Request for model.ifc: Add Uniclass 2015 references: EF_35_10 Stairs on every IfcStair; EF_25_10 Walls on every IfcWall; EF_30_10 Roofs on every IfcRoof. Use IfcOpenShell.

First a look at what the model holds.

```python
import ifcopenshell

model = ifcopenshell.open("model.ifc")
print(model.schema)
print("classifications:", [c.Name for c in model.by_type("IfcClassification")])
for ifc_class in ("IfcDoor", "IfcRoof", "IfcStair", "IfcWall", "IfcWindow"):
    print(ifc_class, len(model.by_type(ifc_class)))
```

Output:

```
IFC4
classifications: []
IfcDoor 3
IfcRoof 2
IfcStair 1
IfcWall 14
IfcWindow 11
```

```python
import ifcopenshell
import ifcopenshell.api.classification

model = ifcopenshell.open("model.ifc")

system = ifcopenshell.api.classification.add_classification(model, classification="Uniclass 2015")

codes = {
    "IfcStair": ("EF_35_10", "Stairs"),
    "IfcWall": ("EF_25_10", "Walls"),
    "IfcRoof": ("EF_30_10", "Roofs"),
}
for ifc_class, (code, name) in codes.items():
    products = model.by_type(ifc_class)
    ifcopenshell.api.classification.add_reference(
        model, products=products, classification=system, identification=code, name=name
    )
    print(code, len(products))

model.write("model_edited.ifc")
```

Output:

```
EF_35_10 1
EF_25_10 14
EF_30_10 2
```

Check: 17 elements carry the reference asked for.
